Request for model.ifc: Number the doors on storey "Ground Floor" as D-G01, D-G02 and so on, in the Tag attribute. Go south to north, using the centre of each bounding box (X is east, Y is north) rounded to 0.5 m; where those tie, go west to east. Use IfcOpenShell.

First a look at what the model holds.

```python
import ifcopenshell
import ifcopenshell.util.element
import ifcopenshell.util.placement

model = ifcopenshell.open("model.ifc")
print(model.schema)
storey = next(s for s in model.by_type("IfcBuildingStorey") if s.Name == "Ground Floor")
doors = [e for e in ifcopenshell.util.element.get_decomposition(storey) if e.is_a("IfcDoor")]
for e in sorted(doors, key=lambda e: e.id()):
    origin = ifcopenshell.util.placement.get_local_placement(e.ObjectPlacement)[:3, 3]
    print(e.id(), e.Tag, e.Name, origin.round(2) + 0.0, sep=" | ")
```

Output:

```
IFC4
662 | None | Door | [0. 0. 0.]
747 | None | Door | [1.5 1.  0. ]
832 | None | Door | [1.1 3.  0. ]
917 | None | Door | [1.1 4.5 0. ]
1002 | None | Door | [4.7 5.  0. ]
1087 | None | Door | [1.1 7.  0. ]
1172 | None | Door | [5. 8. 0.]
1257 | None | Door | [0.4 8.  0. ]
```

```python
import ifcopenshell
import ifcopenshell.geom
import ifcopenshell.util.element
import ifcopenshell.util.shape

model = ifcopenshell.open("model.ifc")
settings = ifcopenshell.geom.settings()
settings.set("use-world-coords", True)


def centre(element):
    shape = ifcopenshell.geom.create_shape(settings, element)
    return ifcopenshell.util.shape.get_bbox_centroid(shape.geometry)


storey = next(s for s in model.by_type("IfcBuildingStorey") if s.Name == "Ground Floor")
doors = [e for e in ifcopenshell.util.element.get_decomposition(storey) if e.is_a("IfcDoor")]

# Insertion points can sit at a corner or the storey origin, so sort by the geometry (in metres).
centres = {e: centre(e) for e in doors}
doors.sort(key=lambda e: (round(centres[e][1] / 0.5), centres[e][0]))

for i, e in enumerate(doors, start=1):
    number = f"D-G{i:02d}"
    e.Tag = number
    print(e.id(), number)

model.write("model_v2.ifc")
```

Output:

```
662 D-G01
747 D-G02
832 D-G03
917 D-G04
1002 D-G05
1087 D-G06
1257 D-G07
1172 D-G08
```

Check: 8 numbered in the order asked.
